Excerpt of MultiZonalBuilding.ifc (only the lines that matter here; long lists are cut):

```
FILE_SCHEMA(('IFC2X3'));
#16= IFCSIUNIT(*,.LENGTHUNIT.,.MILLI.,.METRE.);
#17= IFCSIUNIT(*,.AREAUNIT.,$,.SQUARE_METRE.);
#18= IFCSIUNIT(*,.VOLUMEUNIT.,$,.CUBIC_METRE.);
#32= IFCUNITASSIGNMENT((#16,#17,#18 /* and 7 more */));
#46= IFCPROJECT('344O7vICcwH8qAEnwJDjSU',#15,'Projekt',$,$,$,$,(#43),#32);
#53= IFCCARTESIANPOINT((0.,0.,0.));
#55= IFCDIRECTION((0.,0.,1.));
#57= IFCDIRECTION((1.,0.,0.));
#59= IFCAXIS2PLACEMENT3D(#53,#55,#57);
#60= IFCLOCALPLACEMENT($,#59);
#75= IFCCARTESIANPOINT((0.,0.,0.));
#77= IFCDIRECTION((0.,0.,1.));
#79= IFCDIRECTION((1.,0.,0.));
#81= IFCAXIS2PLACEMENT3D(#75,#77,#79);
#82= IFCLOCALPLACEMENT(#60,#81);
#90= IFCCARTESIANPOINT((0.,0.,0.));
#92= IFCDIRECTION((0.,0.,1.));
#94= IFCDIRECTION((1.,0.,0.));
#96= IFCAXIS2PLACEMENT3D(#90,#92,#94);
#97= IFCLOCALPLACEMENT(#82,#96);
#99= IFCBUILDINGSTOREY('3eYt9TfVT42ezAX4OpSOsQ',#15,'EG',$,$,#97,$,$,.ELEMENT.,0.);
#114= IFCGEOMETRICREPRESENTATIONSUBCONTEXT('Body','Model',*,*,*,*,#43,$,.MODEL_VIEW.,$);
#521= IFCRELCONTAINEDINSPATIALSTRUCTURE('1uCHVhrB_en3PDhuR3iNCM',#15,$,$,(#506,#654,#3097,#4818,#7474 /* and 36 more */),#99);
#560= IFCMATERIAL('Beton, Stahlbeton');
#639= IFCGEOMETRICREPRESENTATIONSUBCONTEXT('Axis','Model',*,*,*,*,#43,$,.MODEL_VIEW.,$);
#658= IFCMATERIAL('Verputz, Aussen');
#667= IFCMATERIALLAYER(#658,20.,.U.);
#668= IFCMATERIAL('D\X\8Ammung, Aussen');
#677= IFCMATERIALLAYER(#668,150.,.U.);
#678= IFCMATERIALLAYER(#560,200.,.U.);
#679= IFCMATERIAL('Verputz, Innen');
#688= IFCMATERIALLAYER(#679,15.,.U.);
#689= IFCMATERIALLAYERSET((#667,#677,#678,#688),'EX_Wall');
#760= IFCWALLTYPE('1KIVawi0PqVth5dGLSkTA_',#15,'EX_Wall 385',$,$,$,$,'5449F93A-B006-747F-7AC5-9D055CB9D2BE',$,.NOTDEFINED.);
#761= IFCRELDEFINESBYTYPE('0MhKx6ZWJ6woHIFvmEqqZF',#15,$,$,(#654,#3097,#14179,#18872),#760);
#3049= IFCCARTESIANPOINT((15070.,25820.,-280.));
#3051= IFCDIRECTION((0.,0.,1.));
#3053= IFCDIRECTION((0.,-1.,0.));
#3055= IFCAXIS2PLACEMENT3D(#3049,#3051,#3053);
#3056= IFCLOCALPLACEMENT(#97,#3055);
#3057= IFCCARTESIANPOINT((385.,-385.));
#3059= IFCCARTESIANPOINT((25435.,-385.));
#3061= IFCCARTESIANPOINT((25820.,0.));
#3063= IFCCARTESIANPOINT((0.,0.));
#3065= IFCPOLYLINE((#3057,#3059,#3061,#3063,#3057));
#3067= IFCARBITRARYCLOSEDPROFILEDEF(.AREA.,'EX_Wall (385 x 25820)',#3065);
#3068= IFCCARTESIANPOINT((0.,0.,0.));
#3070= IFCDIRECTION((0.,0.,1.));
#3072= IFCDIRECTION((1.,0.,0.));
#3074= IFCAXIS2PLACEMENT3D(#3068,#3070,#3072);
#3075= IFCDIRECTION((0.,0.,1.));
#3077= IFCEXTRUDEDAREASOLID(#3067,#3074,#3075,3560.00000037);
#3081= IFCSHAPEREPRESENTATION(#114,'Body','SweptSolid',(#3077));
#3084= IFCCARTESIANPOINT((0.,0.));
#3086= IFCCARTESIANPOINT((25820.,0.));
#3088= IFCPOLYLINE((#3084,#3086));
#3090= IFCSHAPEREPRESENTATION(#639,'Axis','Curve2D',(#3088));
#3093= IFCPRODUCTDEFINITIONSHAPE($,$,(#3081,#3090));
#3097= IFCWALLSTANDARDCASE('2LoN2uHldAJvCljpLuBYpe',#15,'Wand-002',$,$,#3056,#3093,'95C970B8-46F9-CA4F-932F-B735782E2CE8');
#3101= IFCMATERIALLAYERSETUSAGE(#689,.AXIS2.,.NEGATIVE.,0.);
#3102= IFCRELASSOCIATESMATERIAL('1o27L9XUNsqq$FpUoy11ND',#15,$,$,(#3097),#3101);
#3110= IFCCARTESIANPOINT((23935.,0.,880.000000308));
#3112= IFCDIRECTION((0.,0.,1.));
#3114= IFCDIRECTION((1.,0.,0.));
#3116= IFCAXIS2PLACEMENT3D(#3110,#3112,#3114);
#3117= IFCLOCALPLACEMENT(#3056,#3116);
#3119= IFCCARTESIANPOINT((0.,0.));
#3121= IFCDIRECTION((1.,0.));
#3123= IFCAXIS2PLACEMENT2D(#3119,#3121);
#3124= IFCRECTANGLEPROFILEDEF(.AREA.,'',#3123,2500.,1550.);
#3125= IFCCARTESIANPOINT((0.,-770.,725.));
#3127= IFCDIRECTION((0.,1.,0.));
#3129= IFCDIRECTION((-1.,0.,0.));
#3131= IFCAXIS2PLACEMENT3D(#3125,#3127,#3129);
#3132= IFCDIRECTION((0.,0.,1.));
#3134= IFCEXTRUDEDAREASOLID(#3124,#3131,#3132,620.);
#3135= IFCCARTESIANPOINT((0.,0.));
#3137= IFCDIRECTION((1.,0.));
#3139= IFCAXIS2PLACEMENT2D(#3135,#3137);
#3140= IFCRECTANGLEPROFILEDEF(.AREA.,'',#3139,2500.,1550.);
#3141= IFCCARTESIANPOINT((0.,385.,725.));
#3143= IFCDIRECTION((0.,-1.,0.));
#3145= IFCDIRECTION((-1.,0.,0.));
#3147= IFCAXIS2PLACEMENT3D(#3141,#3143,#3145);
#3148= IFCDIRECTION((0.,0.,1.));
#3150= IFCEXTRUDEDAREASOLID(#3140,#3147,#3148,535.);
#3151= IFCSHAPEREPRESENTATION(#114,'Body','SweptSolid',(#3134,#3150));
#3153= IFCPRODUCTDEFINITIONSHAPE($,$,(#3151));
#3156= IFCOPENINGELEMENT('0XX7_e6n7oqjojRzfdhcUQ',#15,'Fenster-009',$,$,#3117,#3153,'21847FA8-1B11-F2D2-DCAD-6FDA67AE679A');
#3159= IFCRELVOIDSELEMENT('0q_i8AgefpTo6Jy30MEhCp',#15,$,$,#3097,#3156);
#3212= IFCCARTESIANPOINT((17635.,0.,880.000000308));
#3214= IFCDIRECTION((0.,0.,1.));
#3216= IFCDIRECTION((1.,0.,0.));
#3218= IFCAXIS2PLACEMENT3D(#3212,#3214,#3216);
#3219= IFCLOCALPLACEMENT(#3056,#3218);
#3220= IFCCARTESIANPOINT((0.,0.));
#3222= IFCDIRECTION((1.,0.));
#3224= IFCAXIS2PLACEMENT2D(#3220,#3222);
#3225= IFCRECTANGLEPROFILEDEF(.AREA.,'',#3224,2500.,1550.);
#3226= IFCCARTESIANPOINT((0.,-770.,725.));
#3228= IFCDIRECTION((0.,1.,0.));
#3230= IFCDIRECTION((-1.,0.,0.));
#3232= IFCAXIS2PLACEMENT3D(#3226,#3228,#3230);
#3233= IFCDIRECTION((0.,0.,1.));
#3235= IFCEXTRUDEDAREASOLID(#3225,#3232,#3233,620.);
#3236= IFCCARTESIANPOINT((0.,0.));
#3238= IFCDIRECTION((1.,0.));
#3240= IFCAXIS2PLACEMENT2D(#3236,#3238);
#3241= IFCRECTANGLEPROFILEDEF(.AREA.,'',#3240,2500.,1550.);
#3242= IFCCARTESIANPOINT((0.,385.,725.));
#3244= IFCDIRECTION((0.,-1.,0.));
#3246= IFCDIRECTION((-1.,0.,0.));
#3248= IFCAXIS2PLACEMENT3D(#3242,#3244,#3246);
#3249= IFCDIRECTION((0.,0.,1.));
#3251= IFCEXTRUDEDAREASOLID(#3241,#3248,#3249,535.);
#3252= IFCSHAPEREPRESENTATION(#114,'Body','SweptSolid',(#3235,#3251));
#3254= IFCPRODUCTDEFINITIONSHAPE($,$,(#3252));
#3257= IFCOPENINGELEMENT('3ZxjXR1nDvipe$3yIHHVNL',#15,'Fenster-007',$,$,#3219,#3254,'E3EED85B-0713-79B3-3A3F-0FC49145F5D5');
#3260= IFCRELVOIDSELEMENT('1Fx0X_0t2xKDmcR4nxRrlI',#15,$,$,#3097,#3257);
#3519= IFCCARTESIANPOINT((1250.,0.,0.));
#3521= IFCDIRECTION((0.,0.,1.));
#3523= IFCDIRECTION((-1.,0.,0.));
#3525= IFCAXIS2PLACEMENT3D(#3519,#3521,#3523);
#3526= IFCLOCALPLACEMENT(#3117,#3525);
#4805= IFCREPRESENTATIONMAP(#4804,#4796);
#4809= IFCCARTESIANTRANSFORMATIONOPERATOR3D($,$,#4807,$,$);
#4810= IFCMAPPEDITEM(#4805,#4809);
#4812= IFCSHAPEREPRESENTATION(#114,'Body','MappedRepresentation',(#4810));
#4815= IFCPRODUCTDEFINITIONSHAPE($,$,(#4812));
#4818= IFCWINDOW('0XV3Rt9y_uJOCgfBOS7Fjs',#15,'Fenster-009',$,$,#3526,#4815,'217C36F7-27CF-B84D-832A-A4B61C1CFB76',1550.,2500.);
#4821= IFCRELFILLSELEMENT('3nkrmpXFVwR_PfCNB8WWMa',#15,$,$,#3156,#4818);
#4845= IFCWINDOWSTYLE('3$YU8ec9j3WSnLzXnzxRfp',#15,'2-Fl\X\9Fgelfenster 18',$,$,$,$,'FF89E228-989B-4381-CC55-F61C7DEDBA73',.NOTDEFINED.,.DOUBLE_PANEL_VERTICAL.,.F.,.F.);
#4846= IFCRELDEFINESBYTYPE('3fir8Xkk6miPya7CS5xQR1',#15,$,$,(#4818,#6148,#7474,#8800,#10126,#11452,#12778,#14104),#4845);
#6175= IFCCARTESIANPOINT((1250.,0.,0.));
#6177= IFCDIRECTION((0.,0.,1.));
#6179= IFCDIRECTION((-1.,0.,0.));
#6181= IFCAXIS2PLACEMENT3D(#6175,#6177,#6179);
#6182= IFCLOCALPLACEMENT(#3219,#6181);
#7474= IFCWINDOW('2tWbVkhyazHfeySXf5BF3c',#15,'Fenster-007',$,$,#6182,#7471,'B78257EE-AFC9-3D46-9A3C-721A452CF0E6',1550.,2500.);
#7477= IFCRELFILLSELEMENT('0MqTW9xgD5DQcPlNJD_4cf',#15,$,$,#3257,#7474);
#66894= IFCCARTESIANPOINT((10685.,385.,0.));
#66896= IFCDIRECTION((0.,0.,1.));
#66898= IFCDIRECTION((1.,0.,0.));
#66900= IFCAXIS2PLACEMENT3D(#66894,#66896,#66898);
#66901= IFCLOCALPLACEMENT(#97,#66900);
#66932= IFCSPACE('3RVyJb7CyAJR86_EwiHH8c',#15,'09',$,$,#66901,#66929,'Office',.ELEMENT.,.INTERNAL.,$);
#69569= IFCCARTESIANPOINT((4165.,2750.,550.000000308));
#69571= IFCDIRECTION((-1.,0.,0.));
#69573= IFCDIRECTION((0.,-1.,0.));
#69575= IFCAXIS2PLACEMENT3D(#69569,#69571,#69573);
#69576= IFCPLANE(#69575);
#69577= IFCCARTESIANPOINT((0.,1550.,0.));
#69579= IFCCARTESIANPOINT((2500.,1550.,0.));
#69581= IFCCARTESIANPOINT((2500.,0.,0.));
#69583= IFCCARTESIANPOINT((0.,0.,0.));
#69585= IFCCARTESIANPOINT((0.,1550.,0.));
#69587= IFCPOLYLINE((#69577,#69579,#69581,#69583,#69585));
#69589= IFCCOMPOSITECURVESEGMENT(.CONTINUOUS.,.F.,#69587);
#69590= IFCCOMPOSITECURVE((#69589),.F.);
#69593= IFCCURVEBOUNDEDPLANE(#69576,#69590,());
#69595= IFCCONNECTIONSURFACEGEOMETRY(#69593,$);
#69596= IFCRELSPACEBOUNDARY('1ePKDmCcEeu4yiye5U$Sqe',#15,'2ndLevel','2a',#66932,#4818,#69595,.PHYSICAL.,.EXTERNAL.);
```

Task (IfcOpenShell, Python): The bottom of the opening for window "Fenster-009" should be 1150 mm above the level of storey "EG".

```python
import numpy as np
import ifcopenshell
import ifcopenshell.api.geometry
import ifcopenshell.geom
import ifcopenshell.util.element
import ifcopenshell.util.placement
import ifcopenshell.util.shape
import ifcopenshell.util.unit

model = ifcopenshell.open("MultiZonalBuilding.ifc")
unit_scale = ifcopenshell.util.unit.calculate_unit_scale(model)

window = model.by_id(4818)
opening = window.FillsVoids[0].RelatingOpeningElement
storey = ifcopenshell.util.element.get_container(window, ifc_class="IfcBuildingStorey")
level = ifcopenshell.util.placement.get_local_placement(storey.ObjectPlacement)[2, 3]

# The opening's origin need not be at the sill, so measure its lowest point.
shape = ifcopenshell.geom.create_shape(ifcopenshell.geom.settings(), opening)
bottom = ifcopenshell.util.shape.get_shape_bottom_elevation(shape, shape.geometry) / unit_scale
dz = level + 1.15 / unit_scale - bottom

shift = np.array([0.0, 0.0, dz])
# The window is placed relative to its opening, so it follows when the opening moves.
matrix = ifcopenshell.util.placement.get_local_placement(opening.ObjectPlacement)
matrix[:3, 3] += shift
ifcopenshell.api.geometry.edit_object_placement(
    model, product=opening, matrix=matrix, is_si=False, should_transform_children=True
)

# Space boundary surfaces are stored in each space's coordinates; move them too.
for rel in window.ProvidesBoundaries:
    if not rel.ConnectionGeometry:
        continue
    surface = rel.ConnectionGeometry.SurfaceOnRelatingElement.BasisSurface
    space_matrix = ifcopenshell.util.placement.get_local_placement(rel.RelatingSpace.ObjectPlacement)
    point = np.array(surface.Position.Location.Coordinates) + space_matrix[:3, :3].T @ shift
    surface.Position = model.createIfcAxis2Placement3D(
        model.createIfcCartesianPoint(point.tolist()), surface.Position.Axis, surface.Position.RefDirection
    )

print(f"moved by {dz * unit_scale:+.3f} m")

model.write("MultiZonalBuilding_v2.ifc")
```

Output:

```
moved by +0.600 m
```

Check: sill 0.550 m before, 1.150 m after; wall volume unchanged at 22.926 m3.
